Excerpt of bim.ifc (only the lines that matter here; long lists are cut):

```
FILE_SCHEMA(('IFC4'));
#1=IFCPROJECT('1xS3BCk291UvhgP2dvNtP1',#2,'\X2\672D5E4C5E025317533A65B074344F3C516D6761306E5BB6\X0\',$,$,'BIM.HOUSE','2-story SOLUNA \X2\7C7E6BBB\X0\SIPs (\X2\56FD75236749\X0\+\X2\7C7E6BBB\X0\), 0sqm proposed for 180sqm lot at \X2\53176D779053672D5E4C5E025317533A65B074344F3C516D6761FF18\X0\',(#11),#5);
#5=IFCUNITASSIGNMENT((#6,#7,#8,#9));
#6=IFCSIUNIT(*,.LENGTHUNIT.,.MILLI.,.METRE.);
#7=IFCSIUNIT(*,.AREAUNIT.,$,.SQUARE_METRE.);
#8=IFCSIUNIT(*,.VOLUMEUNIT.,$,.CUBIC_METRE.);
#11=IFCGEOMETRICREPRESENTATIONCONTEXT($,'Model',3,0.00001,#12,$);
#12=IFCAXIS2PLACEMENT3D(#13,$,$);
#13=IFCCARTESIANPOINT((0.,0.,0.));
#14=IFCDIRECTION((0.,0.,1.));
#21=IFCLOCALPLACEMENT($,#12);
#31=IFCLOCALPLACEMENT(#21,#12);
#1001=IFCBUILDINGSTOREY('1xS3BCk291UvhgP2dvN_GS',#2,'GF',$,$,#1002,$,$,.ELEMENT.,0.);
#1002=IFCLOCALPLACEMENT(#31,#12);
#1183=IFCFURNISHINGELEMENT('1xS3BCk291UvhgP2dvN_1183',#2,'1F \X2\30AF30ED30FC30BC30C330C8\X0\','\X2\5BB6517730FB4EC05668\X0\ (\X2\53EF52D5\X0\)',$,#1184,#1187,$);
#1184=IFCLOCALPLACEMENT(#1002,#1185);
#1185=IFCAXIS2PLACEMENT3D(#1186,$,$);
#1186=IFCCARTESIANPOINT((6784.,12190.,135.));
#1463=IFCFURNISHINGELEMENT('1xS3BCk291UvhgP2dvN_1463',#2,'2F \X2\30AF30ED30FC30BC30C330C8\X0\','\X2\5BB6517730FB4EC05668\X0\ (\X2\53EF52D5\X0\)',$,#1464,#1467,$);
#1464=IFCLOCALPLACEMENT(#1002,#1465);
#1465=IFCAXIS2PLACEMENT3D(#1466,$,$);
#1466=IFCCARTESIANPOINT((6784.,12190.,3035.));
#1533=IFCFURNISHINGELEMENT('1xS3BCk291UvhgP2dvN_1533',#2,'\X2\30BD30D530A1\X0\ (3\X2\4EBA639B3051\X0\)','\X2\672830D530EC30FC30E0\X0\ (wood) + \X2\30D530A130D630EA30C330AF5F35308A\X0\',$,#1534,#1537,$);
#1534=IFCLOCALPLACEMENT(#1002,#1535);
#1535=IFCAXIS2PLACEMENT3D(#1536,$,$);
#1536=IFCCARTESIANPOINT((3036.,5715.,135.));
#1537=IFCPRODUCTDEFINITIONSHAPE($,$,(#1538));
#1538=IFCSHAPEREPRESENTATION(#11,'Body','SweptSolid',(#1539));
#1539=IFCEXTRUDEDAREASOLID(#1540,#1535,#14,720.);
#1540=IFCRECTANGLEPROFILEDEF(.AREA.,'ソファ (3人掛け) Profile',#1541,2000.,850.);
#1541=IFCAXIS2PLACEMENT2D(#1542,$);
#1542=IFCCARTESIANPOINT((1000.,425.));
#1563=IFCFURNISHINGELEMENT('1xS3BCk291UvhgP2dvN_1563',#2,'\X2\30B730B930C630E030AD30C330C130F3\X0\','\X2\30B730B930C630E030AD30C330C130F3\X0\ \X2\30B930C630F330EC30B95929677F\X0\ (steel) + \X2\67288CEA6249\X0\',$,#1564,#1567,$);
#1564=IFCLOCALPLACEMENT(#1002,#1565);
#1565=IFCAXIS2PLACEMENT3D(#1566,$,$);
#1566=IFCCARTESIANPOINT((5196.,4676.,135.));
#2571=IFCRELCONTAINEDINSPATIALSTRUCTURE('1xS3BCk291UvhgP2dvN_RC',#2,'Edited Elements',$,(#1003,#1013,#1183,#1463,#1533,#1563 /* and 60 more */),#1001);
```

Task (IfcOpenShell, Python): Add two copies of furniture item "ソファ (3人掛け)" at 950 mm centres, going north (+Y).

```python
import numpy as np
import ifcopenshell
import ifcopenshell.api.geometry
import ifcopenshell.api.root
import ifcopenshell.util.element
import ifcopenshell.util.placement
import ifcopenshell.util.unit

model = ifcopenshell.open("bim.ifc")
unit_scale = ifcopenshell.util.unit.calculate_unit_scale(model)


def reuse_history(source, copy):
    """copy_class also copies each property set's owner history, people and application; keep the originals."""
    for rel in copy.IsDefinedBy:
        if rel.is_a("IfcRelDefinesByProperties") and (history := rel.RelatingPropertyDefinition.OwnerHistory):
            rel.RelatingPropertyDefinition.OwnerHistory = source.OwnerHistory
            ifcopenshell.util.element.remove_deep2(model, history)


source = model.by_guid("1xS3BCk291UvhgP2dvN_1533")
base = ifcopenshell.util.placement.get_local_placement(source.ObjectPlacement)
step = np.array([0.0, 1.0, 0.0]) * 0.95 / unit_scale

for i in range(1, 3):
    copy = ifcopenshell.api.root.copy_class(model, product=source)
    copy.Representation = ifcopenshell.util.element.copy_deep(
        model, source.Representation, exclude=["IfcGeometricRepresentationContext", "IfcRepresentationMap"]
    )
    reuse_history(source, copy)
    matrix = base.copy()
    matrix[:3, 3] += i * step
    print("added at", matrix[:3, 3].round(3) + 0.0)
    ifcopenshell.api.geometry.edit_object_placement(model, product=copy, matrix=matrix, is_si=False)

model.write("bim_edited.ifc")
```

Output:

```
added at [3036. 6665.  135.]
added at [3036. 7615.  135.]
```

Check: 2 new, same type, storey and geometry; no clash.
